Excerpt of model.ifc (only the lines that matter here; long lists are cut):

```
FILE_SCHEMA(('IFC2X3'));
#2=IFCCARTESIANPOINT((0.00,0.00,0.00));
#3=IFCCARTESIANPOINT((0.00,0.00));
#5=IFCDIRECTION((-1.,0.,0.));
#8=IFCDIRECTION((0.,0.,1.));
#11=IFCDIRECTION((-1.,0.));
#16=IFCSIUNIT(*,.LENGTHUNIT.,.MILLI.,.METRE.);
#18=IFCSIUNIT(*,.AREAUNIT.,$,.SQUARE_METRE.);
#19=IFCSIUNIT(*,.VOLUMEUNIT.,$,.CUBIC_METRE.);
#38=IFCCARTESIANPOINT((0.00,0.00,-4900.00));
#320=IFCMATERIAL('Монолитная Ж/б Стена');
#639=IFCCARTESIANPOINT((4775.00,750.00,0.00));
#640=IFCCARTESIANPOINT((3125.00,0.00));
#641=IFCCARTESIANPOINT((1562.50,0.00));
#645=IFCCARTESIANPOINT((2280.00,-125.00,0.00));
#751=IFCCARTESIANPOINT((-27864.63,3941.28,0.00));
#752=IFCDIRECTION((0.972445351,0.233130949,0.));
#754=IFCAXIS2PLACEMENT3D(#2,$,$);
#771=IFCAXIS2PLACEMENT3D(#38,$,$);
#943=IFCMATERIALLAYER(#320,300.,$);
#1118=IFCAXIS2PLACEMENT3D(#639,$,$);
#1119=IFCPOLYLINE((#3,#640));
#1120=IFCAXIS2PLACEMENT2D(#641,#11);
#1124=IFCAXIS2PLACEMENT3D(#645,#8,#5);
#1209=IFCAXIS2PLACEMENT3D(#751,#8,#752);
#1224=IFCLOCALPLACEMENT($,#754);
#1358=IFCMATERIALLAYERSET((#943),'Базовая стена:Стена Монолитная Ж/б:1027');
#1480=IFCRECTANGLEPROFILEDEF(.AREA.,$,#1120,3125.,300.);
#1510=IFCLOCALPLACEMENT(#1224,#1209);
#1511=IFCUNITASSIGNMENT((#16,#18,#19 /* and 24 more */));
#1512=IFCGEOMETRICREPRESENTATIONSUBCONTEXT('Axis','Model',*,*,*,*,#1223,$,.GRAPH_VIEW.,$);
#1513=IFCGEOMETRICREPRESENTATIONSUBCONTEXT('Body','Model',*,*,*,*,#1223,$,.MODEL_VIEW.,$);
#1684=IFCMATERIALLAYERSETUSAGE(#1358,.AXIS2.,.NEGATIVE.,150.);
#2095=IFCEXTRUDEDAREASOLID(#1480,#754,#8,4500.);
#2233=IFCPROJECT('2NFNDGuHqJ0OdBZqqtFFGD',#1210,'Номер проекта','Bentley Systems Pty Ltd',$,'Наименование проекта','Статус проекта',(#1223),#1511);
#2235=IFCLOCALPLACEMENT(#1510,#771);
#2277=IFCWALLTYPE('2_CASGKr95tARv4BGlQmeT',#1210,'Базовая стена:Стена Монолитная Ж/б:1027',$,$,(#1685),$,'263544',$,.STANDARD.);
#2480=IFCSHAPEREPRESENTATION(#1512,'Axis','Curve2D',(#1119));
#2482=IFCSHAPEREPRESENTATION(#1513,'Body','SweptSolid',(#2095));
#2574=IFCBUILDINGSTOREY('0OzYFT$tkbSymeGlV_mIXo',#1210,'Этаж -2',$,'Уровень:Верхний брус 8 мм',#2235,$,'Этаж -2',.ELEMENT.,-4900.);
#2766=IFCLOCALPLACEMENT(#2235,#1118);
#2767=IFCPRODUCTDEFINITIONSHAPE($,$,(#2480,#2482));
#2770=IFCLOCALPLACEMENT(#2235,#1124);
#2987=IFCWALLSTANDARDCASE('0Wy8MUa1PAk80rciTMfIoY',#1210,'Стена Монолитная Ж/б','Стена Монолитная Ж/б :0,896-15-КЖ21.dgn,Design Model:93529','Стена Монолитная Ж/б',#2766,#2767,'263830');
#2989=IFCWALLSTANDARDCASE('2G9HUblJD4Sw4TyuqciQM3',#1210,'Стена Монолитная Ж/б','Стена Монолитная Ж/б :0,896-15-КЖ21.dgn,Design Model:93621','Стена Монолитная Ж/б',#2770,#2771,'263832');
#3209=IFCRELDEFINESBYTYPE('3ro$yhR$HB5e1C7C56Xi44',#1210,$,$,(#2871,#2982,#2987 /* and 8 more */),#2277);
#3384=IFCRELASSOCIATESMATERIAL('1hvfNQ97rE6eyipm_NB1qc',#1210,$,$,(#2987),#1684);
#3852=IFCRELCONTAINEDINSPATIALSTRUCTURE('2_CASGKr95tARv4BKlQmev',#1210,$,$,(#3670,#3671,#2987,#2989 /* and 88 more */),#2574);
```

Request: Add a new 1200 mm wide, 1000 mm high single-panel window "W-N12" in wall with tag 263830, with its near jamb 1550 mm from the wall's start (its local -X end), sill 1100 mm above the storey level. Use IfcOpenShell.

```python
import numpy as np
import ifcopenshell
import ifcopenshell.api.feature
import ifcopenshell.api.geometry
import ifcopenshell.api.root
import ifcopenshell.api.spatial
import ifcopenshell.api.type
import ifcopenshell.geom
import ifcopenshell.util.element
import ifcopenshell.util.placement
import ifcopenshell.util.representation
import ifcopenshell.util.shape
import ifcopenshell.util.unit

model = ifcopenshell.open("model.ifc")
unit_scale = ifcopenshell.util.unit.calculate_unit_scale(model)
settings = ifcopenshell.geom.settings()


def volume(element):
    """Net volume in cubic metres, openings subtracted."""
    shape = ifcopenshell.geom.create_shape(settings, element)
    return ifcopenshell.util.shape.get_volume(shape.geometry)


wall = model.by_guid("0Wy8MUa1PAk80rciTMfIoY")
storey = ifcopenshell.util.element.get_container(wall, ifc_class="IfcBuildingStorey")
context = ifcopenshell.util.representation.get_context(model, "Model", "Body", "MODEL_VIEW")
before = volume(wall)

width, height, from_end, sill = 1.2, 1, 1.55, 1.1  # metres

# The wall runs along its own X axis, and the end named is its -X end.
wall_shape = ifcopenshell.geom.create_shape(settings, wall)
x, y, z = ifcopenshell.util.shape.get_vertices(wall_shape.geometry).T
start = x.min() + from_end
face, thickness = float(y.min()), float(y.max() - y.min())
wall_matrix = ifcopenshell.util.placement.get_local_placement(wall.ObjectPlacement)
level = ifcopenshell.util.placement.get_local_placement(storey.ObjectPlacement)[2, 3]


def in_wall(x, y):
    """Placement at x, y metres in the wall's axes, at sill height."""
    matrix = wall_matrix.copy()
    matrix[:, 3] = wall_matrix @ np.array([x / unit_scale, y / unit_scale, 0.0, 1.0])
    matrix[2, 3] = level + sill / unit_scale
    return matrix


# Opening: a box that overshoots both wall faces by 50 mm.
opening = ifcopenshell.api.root.create_entity(model, ifc_class="IfcOpeningElement")
box = ifcopenshell.api.geometry.add_wall_representation(
    model, context=context, length=width, height=height, thickness=thickness + 0.1
)
ifcopenshell.api.geometry.assign_representation(model, product=opening, representation=box)
ifcopenshell.api.geometry.edit_object_placement(model, product=opening, matrix=in_wall(start, face - 0.05), is_si=False)
ifcopenshell.api.feature.add_feature(model, feature=opening, element=wall)

window = ifcopenshell.api.root.create_entity(model, ifc_class="IfcWindow", name="W-N12")
window.OverallWidth, window.OverallHeight = width / unit_scale, height / unit_scale
body = ifcopenshell.api.geometry.add_window_representation(
    model,
    context=context,
    overall_width=window.OverallWidth,
    overall_height=window.OverallHeight,
    partition_type="SINGLE_PANEL",
)
ifcopenshell.api.geometry.assign_representation(model, product=window, representation=body)
ifcopenshell.api.spatial.assign_container(model, products=[window], relating_structure=storey)
fills = ifcopenshell.api.feature.add_filling(model, opening=opening, element=window)
fills.OwnerHistory = window.OwnerHistory  # required in IFC2X3

# IFC2X3 keeps the operation on the window style.
style = ifcopenshell.api.root.create_entity(model, ifc_class="IfcWindowStyle", name="W-N12")
style.OperationType, style.ConstructionType = "SINGLE_PANEL", "NOTDEFINED"
style.ParameterTakesPrecedence = style.Sizeable = False
ifcopenshell.api.type.assign_type(model, related_objects=[window], relating_type=style)

# Centre the window in the wall's thickness.
ifcopenshell.api.geometry.edit_object_placement(model, product=window, matrix=in_wall(start, face), is_si=False)
window_shape = ifcopenshell.geom.create_shape(settings, window)
depth = ifcopenshell.util.shape.get_vertices(window_shape.geometry)[:, 1]
offset = face + thickness / 2 - (depth.min() + depth.max()) / 2
ifcopenshell.api.geometry.edit_object_placement(model, product=window, matrix=in_wall(start, offset), is_si=False)

after = volume(wall)

print(f"wall volume {before:.3f} -> {after:.3f} m3")

model.write("model_v2.ifc")
```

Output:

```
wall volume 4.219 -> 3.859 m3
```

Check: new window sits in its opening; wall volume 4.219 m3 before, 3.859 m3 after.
